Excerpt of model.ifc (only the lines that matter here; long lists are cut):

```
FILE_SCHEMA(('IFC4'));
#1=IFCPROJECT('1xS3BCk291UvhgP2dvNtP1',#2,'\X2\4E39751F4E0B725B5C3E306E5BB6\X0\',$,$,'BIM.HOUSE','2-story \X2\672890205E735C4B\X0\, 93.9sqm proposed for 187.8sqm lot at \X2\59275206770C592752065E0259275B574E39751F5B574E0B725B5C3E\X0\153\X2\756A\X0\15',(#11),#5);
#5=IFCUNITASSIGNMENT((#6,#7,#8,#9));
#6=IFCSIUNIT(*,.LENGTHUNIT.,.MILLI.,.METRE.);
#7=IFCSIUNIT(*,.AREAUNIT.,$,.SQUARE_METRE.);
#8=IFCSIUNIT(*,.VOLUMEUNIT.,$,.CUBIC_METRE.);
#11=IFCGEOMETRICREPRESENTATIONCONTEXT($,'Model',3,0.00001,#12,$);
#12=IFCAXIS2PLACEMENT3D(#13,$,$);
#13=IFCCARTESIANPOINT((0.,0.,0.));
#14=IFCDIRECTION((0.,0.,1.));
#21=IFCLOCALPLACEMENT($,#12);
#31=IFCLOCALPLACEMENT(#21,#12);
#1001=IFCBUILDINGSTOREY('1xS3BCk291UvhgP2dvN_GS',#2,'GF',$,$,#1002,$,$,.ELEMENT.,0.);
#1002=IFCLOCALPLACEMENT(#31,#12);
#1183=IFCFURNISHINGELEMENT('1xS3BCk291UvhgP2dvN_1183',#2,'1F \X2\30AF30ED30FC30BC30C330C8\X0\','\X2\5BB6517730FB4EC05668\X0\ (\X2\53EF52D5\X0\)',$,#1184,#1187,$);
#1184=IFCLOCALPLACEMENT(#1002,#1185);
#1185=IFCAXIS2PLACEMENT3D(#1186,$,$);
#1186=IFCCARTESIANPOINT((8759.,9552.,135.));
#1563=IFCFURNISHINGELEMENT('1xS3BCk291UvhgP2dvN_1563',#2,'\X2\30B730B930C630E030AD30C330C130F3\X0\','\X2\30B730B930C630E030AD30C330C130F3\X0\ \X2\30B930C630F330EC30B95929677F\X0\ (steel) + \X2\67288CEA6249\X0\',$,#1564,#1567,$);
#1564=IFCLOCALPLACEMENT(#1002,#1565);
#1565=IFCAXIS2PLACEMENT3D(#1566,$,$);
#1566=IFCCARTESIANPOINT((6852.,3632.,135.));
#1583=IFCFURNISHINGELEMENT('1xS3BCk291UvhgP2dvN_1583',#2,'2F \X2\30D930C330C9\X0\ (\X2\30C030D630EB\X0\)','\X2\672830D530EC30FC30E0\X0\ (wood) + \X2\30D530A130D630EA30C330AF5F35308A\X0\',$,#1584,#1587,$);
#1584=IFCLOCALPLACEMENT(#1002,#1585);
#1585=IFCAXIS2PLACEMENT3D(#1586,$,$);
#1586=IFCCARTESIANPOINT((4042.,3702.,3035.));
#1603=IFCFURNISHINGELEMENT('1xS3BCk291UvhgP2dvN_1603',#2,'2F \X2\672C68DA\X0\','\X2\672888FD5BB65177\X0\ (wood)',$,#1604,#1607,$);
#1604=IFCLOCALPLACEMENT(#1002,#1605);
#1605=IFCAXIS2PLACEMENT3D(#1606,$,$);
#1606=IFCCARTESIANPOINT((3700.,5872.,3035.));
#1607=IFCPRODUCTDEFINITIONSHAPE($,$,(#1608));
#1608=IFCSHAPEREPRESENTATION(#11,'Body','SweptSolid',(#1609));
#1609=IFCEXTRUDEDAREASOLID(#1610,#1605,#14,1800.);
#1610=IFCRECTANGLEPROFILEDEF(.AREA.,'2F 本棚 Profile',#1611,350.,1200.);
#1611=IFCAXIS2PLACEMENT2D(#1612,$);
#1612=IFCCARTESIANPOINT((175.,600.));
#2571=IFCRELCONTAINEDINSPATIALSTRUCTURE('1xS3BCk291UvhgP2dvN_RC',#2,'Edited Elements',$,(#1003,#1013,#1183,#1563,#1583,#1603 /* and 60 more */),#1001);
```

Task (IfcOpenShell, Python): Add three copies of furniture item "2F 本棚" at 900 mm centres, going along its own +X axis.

```python
import ifcopenshell
import ifcopenshell.api.geometry
import ifcopenshell.api.root
import ifcopenshell.util.element
import ifcopenshell.util.placement
import ifcopenshell.util.unit

model = ifcopenshell.open("model.ifc")
unit_scale = ifcopenshell.util.unit.calculate_unit_scale(model)


def reuse_history(source, copy):
    """copy_class also copies each property set's owner history, people and application; keep the originals."""
    for rel in copy.IsDefinedBy:
        if rel.is_a("IfcRelDefinesByProperties") and (history := rel.RelatingPropertyDefinition.OwnerHistory):
            rel.RelatingPropertyDefinition.OwnerHistory = source.OwnerHistory
            ifcopenshell.util.element.remove_deep2(model, history)


source = model.by_guid("1xS3BCk291UvhgP2dvN_1603")
base = ifcopenshell.util.placement.get_local_placement(source.ObjectPlacement)
step = base[:3, 0] * 0.9 / unit_scale

for i in range(1, 4):
    copy = ifcopenshell.api.root.copy_class(model, product=source)
    copy.Representation = ifcopenshell.util.element.copy_deep(
        model, source.Representation, exclude=["IfcGeometricRepresentationContext", "IfcRepresentationMap"]
    )
    reuse_history(source, copy)
    matrix = base.copy()
    matrix[:3, 3] += i * step
    print("added at", matrix[:3, 3].round(3) + 0.0)
    ifcopenshell.api.geometry.edit_object_placement(model, product=copy, matrix=matrix, is_si=False)

model.write("model-out.ifc")
```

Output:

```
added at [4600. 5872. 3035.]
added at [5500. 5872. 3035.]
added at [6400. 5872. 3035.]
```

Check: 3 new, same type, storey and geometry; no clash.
